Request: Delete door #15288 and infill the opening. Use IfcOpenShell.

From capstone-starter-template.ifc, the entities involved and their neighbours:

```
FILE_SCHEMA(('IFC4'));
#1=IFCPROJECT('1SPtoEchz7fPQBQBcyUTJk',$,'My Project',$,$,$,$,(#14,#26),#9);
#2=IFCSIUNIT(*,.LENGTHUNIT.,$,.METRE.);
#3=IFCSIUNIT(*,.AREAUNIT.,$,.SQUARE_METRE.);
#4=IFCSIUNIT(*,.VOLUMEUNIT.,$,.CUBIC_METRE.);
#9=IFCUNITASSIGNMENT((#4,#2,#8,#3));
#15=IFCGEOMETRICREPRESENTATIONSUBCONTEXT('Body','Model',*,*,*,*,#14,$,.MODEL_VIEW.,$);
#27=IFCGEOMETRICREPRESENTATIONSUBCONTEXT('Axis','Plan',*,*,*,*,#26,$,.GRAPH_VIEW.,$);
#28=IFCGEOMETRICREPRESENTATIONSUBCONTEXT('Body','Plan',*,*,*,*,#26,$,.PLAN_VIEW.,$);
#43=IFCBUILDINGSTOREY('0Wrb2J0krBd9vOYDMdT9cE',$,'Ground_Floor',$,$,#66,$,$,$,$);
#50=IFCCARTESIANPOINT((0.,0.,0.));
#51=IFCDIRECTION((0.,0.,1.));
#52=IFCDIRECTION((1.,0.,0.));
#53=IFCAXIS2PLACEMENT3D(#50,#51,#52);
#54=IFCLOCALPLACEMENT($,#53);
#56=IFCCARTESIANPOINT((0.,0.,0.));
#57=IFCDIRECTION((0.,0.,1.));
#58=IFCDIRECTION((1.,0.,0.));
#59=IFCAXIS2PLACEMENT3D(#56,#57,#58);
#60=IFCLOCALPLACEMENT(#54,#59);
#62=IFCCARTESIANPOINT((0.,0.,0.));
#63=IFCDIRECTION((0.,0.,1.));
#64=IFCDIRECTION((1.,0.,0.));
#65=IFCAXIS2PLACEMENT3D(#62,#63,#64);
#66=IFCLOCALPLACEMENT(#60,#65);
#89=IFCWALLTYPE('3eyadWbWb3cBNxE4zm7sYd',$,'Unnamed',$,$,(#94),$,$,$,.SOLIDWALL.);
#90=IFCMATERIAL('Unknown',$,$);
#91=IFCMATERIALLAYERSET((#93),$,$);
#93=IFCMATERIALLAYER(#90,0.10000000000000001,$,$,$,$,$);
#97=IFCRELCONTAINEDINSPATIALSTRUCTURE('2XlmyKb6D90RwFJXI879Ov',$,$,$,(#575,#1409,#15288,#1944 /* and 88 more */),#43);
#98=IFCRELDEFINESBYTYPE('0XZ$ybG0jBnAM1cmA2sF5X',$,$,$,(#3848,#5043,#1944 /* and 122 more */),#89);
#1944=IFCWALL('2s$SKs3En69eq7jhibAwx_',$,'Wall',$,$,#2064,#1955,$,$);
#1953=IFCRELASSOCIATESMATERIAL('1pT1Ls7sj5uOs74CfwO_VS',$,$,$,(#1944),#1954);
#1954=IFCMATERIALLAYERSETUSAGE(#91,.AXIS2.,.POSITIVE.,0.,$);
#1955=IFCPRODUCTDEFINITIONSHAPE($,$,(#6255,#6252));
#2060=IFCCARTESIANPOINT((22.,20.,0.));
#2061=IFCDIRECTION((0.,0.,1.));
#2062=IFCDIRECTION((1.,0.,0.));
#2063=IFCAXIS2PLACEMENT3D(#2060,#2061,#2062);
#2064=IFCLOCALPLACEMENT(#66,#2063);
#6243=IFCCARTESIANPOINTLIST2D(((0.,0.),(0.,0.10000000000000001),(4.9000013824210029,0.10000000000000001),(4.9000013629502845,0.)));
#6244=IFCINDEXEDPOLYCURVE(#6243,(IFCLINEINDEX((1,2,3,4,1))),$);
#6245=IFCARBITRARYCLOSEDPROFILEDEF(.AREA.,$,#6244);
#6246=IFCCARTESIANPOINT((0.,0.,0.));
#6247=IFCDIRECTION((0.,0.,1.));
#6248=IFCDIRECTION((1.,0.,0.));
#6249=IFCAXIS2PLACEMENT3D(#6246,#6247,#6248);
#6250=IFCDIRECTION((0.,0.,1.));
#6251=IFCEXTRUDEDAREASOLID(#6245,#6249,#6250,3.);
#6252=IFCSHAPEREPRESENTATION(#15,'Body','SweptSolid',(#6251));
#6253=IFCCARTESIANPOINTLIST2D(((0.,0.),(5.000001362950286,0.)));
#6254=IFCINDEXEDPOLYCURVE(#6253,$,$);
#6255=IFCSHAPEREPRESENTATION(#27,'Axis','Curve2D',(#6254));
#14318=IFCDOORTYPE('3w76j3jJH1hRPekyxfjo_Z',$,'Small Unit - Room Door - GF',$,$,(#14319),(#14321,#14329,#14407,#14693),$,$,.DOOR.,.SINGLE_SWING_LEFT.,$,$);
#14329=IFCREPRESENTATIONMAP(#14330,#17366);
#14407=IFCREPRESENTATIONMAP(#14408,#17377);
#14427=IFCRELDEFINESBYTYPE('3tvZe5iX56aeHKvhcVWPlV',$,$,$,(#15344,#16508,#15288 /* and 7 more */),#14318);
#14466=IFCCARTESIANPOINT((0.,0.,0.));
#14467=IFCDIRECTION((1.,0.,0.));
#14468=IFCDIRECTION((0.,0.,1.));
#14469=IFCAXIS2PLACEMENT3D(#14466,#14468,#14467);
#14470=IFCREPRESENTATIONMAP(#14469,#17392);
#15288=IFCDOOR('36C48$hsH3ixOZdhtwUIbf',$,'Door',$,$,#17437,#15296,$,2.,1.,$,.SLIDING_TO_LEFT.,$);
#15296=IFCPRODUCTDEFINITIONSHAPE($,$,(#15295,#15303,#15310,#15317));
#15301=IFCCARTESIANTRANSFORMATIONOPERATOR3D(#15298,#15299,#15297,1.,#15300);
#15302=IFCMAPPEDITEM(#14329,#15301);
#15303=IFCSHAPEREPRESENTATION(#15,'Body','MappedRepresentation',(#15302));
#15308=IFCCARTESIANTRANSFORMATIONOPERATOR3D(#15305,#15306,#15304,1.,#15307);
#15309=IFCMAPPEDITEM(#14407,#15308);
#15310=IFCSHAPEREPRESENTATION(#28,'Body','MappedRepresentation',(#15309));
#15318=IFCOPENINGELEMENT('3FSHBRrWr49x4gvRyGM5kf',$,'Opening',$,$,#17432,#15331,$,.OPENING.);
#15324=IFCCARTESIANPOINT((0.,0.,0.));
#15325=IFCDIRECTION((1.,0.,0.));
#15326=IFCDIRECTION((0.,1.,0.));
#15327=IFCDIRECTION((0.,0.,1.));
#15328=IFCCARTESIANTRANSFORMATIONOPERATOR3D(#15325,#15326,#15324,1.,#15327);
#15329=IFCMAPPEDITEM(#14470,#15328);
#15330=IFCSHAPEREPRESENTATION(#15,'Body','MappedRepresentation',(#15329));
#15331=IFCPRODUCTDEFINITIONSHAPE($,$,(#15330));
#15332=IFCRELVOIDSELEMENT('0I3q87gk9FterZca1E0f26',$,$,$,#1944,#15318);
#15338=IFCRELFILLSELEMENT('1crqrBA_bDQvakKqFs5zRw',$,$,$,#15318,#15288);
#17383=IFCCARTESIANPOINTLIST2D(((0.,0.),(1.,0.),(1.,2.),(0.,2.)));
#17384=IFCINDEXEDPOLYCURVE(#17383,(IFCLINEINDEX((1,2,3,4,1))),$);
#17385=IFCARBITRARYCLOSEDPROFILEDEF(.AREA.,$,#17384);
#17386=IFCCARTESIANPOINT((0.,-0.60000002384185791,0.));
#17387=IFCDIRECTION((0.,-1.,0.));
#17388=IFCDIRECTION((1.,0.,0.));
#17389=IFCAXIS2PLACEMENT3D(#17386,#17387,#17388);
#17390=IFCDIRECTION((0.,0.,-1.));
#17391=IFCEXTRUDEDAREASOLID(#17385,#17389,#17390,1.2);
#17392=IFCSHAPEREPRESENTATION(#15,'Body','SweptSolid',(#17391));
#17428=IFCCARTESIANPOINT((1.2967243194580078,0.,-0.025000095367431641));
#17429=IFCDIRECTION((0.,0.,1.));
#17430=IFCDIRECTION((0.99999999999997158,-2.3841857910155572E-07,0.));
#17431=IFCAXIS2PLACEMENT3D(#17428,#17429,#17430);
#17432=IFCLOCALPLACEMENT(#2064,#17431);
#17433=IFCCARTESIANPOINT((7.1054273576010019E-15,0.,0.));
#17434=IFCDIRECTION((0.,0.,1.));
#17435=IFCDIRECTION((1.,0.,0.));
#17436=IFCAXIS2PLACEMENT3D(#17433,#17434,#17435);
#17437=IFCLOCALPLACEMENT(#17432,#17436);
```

```python
import ifcopenshell
import ifcopenshell.api.feature
import ifcopenshell.api.root
import ifcopenshell.geom
import ifcopenshell.util.shape

model = ifcopenshell.open("capstone-starter-template.ifc")
settings = ifcopenshell.geom.settings()


def volume(element):
    """Net volume in cubic metres, openings subtracted."""
    shape = ifcopenshell.geom.create_shape(settings, element)
    return ifcopenshell.util.shape.get_volume(shape.geometry)


door = model.by_guid("36C48$hsH3ixOZdhtwUIbf")
opening = door.FillsVoids[0].RelatingOpeningElement
wall = opening.VoidsElements[0].RelatingBuildingElement
before = volume(wall)

ifcopenshell.api.root.remove_product(model, product=door)
ifcopenshell.api.feature.remove_feature(model, feature=opening)

after = volume(wall)

print(f"wall volume {before:.3f} -> {after:.3f} m3")

model.write("capstone-starter-template_edited.ifc")
```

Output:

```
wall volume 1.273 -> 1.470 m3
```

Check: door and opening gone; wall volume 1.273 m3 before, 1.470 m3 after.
